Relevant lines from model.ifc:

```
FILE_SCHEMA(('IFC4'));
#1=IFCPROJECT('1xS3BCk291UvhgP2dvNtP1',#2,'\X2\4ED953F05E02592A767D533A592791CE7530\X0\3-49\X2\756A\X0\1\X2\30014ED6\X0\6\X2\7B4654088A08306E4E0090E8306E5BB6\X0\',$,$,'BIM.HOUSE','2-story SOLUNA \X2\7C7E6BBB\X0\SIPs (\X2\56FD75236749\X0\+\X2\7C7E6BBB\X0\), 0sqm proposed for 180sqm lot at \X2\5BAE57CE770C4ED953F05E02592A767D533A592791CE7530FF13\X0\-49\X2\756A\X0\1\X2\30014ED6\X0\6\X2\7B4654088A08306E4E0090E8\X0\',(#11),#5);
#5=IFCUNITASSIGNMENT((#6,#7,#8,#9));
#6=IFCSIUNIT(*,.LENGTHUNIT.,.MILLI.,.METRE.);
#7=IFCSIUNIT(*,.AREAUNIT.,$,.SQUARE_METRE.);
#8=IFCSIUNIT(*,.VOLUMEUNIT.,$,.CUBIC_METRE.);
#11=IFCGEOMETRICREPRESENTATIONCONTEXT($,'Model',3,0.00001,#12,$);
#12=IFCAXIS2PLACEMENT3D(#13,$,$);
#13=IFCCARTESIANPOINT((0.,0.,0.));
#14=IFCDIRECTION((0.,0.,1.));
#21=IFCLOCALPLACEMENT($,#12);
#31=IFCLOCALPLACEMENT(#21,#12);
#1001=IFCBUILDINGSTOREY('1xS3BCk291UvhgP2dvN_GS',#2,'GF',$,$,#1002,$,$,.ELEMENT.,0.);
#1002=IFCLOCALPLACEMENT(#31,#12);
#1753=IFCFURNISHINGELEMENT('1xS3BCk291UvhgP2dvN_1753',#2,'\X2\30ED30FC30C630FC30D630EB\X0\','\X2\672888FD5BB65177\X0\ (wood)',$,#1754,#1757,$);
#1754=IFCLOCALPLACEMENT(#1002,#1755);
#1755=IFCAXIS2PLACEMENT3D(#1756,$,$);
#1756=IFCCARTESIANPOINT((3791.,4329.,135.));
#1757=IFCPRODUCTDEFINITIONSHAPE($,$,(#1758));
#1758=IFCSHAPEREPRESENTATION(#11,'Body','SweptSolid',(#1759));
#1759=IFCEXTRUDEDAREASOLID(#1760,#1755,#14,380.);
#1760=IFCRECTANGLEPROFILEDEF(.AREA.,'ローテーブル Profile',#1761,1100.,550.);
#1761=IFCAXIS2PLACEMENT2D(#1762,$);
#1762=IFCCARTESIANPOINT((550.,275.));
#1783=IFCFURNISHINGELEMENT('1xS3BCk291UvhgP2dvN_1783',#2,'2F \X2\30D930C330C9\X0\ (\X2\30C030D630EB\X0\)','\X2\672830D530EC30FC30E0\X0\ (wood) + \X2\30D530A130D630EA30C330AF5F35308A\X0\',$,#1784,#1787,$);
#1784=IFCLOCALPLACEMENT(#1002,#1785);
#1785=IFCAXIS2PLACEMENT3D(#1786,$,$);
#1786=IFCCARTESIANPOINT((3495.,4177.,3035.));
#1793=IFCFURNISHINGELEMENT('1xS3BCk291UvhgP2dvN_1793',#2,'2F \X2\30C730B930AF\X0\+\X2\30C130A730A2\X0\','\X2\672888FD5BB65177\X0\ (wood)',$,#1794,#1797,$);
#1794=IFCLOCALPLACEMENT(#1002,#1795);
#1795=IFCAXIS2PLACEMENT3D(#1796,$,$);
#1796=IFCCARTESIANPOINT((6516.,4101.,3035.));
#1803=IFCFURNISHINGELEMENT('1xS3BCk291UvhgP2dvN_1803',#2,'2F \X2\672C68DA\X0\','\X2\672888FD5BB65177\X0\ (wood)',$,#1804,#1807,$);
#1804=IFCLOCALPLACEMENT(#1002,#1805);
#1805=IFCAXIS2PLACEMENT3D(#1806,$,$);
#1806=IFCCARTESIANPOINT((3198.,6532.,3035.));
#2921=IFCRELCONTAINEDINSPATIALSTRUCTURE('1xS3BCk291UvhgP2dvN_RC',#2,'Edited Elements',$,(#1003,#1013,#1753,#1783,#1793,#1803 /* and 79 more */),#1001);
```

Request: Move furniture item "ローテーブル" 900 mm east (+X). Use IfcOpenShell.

```python
import ifcopenshell
import ifcopenshell.api.geometry
import ifcopenshell.util.placement

model = ifcopenshell.open("model.ifc")

item = model.by_id(1753)
matrix = ifcopenshell.util.placement.get_local_placement(item.ObjectPlacement)
matrix[0, 3] += 900.0
ifcopenshell.api.geometry.edit_object_placement(model, product=item, matrix=matrix, is_si=False)

print(ifcopenshell.util.placement.get_local_placement(item.ObjectPlacement).round(3) + 0.0)

model.write("model_v2.ifc")
```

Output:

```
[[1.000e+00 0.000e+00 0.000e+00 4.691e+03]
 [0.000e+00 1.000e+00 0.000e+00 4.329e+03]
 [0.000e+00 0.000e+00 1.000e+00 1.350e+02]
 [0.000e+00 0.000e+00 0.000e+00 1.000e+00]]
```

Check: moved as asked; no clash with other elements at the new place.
